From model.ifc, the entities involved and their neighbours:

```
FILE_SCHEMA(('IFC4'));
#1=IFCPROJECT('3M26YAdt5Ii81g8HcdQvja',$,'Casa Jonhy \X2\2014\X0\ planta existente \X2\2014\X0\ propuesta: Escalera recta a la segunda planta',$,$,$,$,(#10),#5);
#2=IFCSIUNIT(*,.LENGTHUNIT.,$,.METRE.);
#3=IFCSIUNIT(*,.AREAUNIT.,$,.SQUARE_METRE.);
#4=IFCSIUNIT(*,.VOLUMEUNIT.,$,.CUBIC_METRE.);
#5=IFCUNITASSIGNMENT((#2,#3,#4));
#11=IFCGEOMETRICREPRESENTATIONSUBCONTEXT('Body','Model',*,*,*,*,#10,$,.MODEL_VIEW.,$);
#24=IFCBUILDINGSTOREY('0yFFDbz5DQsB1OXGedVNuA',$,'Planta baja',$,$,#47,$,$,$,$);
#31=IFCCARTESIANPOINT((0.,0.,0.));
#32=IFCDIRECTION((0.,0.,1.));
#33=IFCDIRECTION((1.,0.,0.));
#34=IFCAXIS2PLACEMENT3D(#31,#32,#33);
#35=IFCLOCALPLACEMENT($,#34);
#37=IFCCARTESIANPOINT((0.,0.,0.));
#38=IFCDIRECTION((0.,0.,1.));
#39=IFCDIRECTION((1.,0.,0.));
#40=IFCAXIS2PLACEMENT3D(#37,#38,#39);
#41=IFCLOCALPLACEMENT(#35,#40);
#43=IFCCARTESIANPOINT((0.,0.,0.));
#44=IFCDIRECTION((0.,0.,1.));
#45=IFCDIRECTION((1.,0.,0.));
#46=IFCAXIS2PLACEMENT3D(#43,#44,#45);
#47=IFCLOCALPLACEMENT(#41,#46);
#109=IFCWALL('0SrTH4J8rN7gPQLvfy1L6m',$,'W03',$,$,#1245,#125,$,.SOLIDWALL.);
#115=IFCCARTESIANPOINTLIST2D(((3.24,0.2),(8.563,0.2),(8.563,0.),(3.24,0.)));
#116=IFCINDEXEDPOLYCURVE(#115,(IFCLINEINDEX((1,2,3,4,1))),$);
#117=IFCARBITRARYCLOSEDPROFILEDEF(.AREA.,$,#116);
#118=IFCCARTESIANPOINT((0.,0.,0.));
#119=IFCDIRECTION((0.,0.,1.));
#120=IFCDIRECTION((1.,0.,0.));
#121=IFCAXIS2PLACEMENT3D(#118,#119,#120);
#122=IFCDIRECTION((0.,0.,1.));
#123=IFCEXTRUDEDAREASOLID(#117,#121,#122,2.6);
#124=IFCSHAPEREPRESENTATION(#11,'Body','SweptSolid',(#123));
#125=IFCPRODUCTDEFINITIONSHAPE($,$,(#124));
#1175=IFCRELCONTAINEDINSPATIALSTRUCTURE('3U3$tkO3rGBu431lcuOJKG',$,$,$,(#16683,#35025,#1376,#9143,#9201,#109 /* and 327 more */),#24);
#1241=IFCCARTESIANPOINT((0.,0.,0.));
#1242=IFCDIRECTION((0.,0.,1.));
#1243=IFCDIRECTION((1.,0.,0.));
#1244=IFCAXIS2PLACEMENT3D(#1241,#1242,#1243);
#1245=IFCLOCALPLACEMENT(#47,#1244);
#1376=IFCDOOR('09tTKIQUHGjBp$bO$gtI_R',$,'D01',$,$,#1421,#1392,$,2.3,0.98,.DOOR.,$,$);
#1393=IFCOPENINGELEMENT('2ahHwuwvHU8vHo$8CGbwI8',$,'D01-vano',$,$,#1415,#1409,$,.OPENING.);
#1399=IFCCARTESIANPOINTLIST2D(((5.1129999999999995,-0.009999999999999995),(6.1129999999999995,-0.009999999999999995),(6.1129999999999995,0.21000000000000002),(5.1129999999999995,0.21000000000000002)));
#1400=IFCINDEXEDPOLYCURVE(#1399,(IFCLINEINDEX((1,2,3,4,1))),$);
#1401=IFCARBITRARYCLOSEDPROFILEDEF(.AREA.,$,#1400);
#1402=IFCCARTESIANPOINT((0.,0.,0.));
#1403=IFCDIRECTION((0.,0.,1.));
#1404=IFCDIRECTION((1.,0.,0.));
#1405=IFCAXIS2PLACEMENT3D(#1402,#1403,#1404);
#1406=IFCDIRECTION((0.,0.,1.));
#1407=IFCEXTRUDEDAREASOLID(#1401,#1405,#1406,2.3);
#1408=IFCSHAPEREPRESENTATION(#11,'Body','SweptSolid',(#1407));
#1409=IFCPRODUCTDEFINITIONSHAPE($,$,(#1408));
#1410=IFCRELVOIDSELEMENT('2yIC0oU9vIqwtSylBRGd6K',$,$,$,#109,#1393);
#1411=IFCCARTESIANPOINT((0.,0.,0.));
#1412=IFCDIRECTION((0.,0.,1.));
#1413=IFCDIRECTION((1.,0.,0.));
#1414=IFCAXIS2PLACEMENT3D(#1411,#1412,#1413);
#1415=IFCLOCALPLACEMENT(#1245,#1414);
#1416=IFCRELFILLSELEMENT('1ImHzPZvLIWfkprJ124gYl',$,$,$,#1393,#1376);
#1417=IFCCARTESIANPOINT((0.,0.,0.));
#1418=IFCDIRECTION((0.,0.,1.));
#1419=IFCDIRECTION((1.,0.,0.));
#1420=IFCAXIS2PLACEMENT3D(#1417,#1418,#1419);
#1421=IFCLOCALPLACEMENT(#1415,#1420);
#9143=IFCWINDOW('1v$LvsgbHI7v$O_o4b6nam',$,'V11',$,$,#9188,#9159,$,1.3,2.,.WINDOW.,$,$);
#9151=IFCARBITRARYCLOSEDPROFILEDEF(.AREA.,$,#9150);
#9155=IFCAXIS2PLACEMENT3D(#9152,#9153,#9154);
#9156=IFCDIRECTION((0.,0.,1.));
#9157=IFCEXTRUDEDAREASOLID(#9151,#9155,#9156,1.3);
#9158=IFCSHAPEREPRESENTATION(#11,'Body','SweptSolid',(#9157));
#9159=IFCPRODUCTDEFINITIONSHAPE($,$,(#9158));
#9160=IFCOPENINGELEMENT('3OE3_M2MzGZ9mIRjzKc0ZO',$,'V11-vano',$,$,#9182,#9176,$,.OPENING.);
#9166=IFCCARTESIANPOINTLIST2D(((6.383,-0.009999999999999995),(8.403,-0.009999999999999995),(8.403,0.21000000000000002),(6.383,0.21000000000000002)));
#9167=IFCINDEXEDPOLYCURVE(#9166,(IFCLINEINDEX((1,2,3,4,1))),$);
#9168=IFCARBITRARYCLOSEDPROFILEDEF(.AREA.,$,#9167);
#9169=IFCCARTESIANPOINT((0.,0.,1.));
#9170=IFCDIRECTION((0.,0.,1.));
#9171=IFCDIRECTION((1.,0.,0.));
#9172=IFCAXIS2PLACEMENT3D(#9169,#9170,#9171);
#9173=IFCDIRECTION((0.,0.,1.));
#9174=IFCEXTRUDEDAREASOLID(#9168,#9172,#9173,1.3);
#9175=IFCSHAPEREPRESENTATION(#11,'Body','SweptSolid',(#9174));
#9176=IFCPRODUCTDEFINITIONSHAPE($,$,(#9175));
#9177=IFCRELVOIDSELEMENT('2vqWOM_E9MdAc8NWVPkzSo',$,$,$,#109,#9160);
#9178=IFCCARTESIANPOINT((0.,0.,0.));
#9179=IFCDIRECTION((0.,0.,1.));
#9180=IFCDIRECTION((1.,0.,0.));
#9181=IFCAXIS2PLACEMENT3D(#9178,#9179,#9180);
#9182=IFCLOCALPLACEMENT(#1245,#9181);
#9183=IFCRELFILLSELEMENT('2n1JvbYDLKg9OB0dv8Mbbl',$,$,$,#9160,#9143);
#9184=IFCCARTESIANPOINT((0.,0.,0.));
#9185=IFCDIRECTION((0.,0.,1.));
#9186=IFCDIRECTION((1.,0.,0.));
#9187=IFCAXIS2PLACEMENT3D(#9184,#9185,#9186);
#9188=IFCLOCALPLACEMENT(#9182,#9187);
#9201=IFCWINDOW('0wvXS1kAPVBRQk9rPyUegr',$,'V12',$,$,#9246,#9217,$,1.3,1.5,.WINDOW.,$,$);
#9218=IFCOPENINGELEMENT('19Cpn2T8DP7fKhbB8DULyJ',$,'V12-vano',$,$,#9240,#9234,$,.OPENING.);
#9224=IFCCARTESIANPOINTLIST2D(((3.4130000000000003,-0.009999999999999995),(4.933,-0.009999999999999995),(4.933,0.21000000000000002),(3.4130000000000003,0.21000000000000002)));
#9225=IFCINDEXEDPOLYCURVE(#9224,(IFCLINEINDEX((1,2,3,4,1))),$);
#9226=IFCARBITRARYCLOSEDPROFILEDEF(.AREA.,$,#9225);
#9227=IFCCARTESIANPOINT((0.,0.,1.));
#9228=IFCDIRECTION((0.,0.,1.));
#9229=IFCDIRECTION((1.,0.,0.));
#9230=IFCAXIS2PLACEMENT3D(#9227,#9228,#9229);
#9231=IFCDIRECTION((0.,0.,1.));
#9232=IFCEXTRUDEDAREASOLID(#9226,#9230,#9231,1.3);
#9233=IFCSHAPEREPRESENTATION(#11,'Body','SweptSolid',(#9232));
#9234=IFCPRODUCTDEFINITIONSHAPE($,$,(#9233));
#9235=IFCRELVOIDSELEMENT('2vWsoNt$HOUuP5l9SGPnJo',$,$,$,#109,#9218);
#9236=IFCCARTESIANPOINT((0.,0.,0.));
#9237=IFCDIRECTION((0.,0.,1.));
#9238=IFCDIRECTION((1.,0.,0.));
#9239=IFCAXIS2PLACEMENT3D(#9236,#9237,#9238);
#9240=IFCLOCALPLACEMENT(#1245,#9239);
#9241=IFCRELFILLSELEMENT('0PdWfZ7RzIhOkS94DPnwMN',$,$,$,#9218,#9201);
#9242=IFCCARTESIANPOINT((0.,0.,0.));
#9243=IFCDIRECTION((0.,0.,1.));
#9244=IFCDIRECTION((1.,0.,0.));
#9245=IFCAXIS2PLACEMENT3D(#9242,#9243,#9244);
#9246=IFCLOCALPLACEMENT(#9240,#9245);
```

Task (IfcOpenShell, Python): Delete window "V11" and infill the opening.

```python
import ifcopenshell
import ifcopenshell.api.feature
import ifcopenshell.api.root
import ifcopenshell.geom
import ifcopenshell.util.shape

model = ifcopenshell.open("model.ifc")
settings = ifcopenshell.geom.settings()


def volume(element):
    """Net volume in cubic metres, openings subtracted."""
    shape = ifcopenshell.geom.create_shape(settings, element)
    return ifcopenshell.util.shape.get_volume(shape.geometry)


window = model.by_id(9143)
opening = window.FillsVoids[0].RelatingOpeningElement
wall = opening.VoidsElements[0].RelatingBuildingElement
before = volume(wall)

ifcopenshell.api.root.remove_product(model, product=window)
ifcopenshell.api.feature.remove_feature(model, feature=opening)

after = volume(wall)

print(f"wall volume {before:.3f} -> {after:.3f} m3")

model.write("model_rev.ifc")
```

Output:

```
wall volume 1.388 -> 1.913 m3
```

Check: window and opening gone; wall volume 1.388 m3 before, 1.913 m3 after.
